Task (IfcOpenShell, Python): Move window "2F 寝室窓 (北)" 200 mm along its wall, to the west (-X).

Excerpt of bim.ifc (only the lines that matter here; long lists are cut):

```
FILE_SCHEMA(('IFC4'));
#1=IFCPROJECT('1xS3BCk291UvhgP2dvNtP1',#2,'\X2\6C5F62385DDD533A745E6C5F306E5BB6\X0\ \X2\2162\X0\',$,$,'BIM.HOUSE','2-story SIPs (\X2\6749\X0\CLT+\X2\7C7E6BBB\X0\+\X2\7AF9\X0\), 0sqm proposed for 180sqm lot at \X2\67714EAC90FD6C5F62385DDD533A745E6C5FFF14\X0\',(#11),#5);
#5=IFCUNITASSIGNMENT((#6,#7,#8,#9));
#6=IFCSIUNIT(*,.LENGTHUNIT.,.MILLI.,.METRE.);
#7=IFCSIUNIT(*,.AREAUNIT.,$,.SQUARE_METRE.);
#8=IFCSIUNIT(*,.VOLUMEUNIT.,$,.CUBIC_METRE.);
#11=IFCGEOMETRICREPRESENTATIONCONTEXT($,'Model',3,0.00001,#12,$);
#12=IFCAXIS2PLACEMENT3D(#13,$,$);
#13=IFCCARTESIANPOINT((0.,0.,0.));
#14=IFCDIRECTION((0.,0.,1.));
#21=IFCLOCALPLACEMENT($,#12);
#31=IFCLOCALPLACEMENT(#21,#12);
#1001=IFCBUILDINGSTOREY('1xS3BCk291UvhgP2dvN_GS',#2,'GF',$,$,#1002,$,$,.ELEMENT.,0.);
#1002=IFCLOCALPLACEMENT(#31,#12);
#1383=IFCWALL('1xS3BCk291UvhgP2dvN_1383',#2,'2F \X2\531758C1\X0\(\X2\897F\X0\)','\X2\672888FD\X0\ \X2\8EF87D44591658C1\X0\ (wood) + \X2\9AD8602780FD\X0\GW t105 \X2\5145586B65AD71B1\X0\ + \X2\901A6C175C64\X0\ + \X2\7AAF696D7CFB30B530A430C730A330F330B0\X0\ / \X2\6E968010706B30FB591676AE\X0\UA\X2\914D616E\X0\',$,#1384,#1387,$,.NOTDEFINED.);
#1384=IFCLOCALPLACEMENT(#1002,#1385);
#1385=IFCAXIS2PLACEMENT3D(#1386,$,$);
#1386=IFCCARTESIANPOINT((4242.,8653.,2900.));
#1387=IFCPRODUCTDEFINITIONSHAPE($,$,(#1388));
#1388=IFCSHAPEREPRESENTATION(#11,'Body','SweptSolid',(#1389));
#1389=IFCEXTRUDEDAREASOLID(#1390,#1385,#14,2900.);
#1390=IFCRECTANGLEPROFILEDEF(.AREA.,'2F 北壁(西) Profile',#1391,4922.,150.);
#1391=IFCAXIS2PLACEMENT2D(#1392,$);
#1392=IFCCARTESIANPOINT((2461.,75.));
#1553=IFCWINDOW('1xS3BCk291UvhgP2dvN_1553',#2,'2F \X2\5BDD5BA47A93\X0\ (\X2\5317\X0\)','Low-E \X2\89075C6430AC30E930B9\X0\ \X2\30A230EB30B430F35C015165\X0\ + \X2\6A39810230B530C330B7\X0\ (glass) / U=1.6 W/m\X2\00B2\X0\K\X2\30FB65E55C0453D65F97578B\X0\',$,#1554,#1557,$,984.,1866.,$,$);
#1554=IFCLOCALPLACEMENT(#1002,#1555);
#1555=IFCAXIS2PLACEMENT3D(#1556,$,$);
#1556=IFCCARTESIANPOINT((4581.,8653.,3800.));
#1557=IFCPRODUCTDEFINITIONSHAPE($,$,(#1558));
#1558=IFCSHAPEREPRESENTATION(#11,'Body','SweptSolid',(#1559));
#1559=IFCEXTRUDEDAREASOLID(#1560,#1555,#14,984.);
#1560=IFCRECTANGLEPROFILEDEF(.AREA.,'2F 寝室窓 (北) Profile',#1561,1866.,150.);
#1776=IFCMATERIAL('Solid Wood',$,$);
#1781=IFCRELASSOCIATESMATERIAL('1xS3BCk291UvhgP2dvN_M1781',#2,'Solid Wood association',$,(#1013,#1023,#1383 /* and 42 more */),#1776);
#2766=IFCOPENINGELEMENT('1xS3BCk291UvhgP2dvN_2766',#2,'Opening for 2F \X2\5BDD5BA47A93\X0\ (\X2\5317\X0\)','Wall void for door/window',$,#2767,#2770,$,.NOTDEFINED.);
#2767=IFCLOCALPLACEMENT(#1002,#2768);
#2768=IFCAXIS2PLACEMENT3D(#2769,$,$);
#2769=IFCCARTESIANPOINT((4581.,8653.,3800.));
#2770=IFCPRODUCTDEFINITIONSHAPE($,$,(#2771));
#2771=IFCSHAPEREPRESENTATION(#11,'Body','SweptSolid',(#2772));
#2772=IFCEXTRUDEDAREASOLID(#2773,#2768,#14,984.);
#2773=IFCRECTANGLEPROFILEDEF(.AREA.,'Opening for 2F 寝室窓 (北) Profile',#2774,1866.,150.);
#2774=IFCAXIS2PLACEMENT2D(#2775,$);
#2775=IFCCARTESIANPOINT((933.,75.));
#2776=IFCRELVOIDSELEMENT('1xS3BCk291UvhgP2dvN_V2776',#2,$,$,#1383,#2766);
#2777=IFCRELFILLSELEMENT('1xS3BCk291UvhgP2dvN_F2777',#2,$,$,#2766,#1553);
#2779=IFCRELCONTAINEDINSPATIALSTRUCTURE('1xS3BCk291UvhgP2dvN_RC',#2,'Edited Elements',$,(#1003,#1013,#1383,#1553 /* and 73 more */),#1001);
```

```python
import ifcopenshell
import ifcopenshell.api.geometry
import ifcopenshell.util.placement

model = ifcopenshell.open("bim.ifc")

window = model.by_guid("1xS3BCk291UvhgP2dvN_1553")
opening = window.FillsVoids[0].RelatingOpeningElement
wall = opening.VoidsElements[0].RelatingBuildingElement

wall_matrix = ifcopenshell.util.placement.get_local_placement(wall.ObjectPlacement)
shift = wall_matrix[:3, 0] * -200.0
before = ifcopenshell.util.placement.get_local_placement(window.ObjectPlacement)[:3, 3].copy()

# The window is not placed relative to its opening, so move both.
for product in (opening, window):
    matrix = ifcopenshell.util.placement.get_local_placement(product.ObjectPlacement)
    matrix[:3, 3] += shift
    ifcopenshell.api.geometry.edit_object_placement(model, product=product, matrix=matrix, is_si=False)

after = ifcopenshell.util.placement.get_local_placement(window.ObjectPlacement)[:3, 3]
print("window moved by", (after - before).round(3) + 0.0)

model.write("bim_updated.ifc")
```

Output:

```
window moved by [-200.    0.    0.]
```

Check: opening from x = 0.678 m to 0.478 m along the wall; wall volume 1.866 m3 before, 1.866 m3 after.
